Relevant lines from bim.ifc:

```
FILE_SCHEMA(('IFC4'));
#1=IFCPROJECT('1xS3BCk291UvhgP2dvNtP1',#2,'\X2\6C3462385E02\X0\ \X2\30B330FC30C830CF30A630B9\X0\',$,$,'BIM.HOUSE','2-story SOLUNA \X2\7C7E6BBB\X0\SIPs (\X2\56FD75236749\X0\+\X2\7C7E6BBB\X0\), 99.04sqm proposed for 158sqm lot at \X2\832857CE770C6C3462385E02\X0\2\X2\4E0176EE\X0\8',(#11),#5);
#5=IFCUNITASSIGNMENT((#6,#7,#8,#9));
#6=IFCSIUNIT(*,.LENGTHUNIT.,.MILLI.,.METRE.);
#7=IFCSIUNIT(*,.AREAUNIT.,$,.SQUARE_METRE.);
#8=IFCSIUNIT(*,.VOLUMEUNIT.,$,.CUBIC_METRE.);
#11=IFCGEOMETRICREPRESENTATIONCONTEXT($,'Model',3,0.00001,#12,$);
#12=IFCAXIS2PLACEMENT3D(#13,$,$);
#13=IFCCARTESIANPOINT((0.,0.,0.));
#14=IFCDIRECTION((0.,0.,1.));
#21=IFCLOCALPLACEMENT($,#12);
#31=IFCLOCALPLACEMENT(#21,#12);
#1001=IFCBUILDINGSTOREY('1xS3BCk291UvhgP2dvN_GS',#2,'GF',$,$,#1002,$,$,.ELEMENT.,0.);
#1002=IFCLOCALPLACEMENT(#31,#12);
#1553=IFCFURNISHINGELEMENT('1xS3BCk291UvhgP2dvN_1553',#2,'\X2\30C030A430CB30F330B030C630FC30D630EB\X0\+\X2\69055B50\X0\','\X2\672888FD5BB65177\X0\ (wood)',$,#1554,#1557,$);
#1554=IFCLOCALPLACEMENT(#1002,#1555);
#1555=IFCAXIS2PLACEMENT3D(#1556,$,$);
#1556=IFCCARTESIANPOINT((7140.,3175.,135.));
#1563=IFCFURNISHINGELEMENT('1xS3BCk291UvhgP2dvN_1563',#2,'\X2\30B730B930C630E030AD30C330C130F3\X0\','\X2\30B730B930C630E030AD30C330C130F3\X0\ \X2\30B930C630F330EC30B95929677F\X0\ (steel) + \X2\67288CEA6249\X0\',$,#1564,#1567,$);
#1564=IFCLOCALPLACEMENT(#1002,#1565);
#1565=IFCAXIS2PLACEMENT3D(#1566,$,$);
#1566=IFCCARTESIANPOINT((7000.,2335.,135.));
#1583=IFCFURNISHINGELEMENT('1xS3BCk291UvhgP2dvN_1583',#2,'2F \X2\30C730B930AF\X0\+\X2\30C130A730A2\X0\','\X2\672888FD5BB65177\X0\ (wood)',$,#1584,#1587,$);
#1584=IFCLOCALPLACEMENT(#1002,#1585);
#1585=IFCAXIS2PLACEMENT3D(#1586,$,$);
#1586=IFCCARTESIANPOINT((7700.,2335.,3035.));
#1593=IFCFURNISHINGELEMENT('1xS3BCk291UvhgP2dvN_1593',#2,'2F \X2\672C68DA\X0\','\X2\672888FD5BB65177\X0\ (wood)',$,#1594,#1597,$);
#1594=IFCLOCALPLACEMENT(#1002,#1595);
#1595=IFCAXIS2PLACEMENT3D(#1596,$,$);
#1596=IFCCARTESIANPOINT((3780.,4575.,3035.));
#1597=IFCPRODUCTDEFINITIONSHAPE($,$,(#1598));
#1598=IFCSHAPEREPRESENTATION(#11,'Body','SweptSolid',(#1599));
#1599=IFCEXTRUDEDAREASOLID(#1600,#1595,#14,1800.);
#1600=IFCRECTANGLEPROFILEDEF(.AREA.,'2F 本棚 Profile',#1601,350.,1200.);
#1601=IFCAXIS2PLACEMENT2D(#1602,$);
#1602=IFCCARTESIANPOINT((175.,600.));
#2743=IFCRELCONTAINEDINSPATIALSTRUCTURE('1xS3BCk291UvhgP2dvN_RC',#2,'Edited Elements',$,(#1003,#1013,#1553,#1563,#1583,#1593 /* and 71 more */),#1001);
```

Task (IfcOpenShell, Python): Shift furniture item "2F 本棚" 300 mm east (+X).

```python
import ifcopenshell
import ifcopenshell.api.geometry
import ifcopenshell.util.placement
import ifcopenshell.util.unit

model = ifcopenshell.open("bim.ifc")
unit_scale = ifcopenshell.util.unit.calculate_unit_scale(model)

item = model.by_id(1593)
matrix = ifcopenshell.util.placement.get_local_placement(item.ObjectPlacement)
matrix[0, 3] += 0.3 / unit_scale
ifcopenshell.api.geometry.edit_object_placement(model, product=item, matrix=matrix, is_si=False)

print(ifcopenshell.util.placement.get_local_placement(item.ObjectPlacement).round(3) + 0.0)

model.write("bim_v2.ifc")
```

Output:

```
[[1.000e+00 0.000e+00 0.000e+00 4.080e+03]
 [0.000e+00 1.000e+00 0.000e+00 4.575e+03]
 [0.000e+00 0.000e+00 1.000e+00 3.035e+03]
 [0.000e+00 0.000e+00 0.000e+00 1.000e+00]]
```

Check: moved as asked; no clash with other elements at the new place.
